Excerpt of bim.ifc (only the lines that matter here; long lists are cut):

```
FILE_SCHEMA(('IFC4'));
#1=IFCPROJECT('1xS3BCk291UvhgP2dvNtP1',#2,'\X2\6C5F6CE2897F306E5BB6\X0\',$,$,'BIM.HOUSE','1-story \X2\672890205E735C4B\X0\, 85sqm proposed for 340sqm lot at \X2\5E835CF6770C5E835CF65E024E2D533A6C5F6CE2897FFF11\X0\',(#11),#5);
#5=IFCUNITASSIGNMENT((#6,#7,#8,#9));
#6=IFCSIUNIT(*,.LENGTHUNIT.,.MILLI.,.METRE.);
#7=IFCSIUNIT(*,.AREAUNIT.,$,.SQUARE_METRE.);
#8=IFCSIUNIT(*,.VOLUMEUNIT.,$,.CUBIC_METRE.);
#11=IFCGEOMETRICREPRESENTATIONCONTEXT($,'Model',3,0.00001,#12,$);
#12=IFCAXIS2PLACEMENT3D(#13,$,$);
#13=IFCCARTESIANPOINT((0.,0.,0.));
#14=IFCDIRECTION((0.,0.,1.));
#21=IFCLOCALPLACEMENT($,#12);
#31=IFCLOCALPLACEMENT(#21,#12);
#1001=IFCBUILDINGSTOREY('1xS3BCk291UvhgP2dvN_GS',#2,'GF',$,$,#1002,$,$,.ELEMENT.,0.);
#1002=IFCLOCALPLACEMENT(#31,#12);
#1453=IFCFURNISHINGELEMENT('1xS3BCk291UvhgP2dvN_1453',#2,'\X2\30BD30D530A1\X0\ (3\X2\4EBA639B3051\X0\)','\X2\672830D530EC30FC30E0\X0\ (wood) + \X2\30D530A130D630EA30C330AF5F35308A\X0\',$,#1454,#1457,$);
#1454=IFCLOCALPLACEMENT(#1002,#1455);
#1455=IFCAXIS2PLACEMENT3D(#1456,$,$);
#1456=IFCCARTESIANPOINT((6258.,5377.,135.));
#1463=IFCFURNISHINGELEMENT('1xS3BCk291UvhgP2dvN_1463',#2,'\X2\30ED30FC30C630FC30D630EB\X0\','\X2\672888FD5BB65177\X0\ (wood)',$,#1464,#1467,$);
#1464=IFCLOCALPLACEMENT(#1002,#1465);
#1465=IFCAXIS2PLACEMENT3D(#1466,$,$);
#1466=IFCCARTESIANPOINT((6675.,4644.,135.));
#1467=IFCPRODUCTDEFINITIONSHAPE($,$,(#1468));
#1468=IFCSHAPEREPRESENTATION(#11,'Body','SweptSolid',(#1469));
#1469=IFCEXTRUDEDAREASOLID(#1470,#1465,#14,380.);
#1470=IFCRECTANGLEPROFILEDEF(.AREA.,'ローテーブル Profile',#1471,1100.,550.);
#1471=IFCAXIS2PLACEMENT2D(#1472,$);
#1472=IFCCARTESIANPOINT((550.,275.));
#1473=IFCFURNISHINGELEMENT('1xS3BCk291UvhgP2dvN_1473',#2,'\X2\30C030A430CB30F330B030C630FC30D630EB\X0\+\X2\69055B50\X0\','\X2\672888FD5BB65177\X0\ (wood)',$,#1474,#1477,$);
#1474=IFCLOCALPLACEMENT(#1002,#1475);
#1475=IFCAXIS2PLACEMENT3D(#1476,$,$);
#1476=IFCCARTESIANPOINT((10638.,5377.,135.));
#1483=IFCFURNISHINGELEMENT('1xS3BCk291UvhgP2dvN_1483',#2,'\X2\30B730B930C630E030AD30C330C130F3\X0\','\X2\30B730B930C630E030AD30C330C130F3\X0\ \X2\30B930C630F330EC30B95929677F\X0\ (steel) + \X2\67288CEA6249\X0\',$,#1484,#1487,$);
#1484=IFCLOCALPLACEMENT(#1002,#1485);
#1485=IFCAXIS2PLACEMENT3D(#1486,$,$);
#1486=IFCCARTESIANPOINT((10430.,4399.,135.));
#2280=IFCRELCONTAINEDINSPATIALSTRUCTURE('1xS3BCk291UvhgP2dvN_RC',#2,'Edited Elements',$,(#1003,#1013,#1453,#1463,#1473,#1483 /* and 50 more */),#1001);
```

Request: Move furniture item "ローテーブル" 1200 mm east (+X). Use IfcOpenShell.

```python
import ifcopenshell
import ifcopenshell.api.geometry
import ifcopenshell.util.placement
import ifcopenshell.util.unit

model = ifcopenshell.open("bim.ifc")
unit_scale = ifcopenshell.util.unit.calculate_unit_scale(model)

item = model.by_guid("1xS3BCk291UvhgP2dvN_1463")
matrix = ifcopenshell.util.placement.get_local_placement(item.ObjectPlacement)
matrix[0, 3] += 1.2 / unit_scale
ifcopenshell.api.geometry.edit_object_placement(model, product=item, matrix=matrix, is_si=False)

print(ifcopenshell.util.placement.get_local_placement(item.ObjectPlacement).round(3) + 0.0)

model.write("bim_updated.ifc")
```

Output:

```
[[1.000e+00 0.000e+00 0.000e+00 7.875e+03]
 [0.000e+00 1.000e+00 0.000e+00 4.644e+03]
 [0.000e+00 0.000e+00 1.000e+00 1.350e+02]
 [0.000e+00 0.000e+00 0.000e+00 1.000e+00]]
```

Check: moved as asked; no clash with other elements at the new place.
